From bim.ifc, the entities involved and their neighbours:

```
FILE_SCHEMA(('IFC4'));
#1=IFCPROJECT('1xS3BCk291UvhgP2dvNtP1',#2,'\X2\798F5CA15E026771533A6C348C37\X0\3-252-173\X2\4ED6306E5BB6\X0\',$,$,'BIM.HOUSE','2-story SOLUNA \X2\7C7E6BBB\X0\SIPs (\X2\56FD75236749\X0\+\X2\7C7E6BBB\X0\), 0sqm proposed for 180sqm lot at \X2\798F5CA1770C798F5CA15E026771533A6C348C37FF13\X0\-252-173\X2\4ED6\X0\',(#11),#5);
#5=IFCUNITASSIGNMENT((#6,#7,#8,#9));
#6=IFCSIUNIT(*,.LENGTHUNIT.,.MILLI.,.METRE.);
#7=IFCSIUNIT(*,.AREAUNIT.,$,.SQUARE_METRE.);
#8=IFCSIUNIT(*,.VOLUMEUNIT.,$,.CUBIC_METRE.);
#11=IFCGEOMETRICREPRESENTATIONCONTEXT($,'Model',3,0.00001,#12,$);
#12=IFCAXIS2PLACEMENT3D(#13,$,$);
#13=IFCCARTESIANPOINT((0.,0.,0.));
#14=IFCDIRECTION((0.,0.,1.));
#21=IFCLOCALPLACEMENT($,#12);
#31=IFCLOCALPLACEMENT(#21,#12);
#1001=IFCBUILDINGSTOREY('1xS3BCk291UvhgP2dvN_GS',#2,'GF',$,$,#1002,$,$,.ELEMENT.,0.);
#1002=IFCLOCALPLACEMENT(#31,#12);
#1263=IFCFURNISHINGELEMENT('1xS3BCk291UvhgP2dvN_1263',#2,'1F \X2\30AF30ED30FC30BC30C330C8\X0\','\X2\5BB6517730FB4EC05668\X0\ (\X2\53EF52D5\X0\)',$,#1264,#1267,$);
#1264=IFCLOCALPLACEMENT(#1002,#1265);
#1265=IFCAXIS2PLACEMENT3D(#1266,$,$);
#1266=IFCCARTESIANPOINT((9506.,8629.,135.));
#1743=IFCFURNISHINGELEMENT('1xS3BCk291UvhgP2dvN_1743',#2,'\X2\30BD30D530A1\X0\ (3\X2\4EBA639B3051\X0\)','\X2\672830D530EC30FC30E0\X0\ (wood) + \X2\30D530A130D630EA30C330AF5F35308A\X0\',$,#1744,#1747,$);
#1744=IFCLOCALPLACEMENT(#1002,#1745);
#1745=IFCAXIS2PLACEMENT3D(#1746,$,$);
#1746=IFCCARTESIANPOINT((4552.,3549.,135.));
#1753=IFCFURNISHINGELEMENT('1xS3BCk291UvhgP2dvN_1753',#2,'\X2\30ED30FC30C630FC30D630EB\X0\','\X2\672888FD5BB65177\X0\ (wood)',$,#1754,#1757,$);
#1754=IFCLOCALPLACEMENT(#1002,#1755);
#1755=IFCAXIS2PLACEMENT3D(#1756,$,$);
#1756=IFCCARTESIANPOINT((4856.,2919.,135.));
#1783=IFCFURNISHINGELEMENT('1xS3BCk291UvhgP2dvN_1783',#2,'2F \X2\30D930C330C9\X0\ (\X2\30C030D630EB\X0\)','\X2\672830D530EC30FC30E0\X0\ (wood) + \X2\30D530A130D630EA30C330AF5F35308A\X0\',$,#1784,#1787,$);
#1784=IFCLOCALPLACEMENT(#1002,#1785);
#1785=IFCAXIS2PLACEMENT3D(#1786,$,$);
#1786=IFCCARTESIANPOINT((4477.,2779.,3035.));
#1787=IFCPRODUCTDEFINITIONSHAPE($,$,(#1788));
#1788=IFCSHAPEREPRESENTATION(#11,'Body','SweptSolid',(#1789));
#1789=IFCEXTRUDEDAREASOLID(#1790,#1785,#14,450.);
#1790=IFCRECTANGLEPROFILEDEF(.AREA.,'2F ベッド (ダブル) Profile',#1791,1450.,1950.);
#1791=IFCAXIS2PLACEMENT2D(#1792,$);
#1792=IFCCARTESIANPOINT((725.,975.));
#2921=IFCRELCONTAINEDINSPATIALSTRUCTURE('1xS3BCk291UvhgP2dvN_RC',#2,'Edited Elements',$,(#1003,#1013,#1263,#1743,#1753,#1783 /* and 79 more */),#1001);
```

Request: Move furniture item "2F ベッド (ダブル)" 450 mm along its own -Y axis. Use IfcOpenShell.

```python
import ifcopenshell
import ifcopenshell.api.geometry
import ifcopenshell.util.placement
import ifcopenshell.util.unit

model = ifcopenshell.open("bim.ifc")
unit_scale = ifcopenshell.util.unit.calculate_unit_scale(model)

item = model.by_guid("1xS3BCk291UvhgP2dvN_1783")
matrix = ifcopenshell.util.placement.get_local_placement(item.ObjectPlacement)
matrix[:3, 3] -= matrix[:3, 1] * 0.45 / unit_scale
ifcopenshell.api.geometry.edit_object_placement(model, product=item, matrix=matrix, is_si=False)

print(ifcopenshell.util.placement.get_local_placement(item.ObjectPlacement).round(3) + 0.0)

model.write("bim_rev.ifc")
```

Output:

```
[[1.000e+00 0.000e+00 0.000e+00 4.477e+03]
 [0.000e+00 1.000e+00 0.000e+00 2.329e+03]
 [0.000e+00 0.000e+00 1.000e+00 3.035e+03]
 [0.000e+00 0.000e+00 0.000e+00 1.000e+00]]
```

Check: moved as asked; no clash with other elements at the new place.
